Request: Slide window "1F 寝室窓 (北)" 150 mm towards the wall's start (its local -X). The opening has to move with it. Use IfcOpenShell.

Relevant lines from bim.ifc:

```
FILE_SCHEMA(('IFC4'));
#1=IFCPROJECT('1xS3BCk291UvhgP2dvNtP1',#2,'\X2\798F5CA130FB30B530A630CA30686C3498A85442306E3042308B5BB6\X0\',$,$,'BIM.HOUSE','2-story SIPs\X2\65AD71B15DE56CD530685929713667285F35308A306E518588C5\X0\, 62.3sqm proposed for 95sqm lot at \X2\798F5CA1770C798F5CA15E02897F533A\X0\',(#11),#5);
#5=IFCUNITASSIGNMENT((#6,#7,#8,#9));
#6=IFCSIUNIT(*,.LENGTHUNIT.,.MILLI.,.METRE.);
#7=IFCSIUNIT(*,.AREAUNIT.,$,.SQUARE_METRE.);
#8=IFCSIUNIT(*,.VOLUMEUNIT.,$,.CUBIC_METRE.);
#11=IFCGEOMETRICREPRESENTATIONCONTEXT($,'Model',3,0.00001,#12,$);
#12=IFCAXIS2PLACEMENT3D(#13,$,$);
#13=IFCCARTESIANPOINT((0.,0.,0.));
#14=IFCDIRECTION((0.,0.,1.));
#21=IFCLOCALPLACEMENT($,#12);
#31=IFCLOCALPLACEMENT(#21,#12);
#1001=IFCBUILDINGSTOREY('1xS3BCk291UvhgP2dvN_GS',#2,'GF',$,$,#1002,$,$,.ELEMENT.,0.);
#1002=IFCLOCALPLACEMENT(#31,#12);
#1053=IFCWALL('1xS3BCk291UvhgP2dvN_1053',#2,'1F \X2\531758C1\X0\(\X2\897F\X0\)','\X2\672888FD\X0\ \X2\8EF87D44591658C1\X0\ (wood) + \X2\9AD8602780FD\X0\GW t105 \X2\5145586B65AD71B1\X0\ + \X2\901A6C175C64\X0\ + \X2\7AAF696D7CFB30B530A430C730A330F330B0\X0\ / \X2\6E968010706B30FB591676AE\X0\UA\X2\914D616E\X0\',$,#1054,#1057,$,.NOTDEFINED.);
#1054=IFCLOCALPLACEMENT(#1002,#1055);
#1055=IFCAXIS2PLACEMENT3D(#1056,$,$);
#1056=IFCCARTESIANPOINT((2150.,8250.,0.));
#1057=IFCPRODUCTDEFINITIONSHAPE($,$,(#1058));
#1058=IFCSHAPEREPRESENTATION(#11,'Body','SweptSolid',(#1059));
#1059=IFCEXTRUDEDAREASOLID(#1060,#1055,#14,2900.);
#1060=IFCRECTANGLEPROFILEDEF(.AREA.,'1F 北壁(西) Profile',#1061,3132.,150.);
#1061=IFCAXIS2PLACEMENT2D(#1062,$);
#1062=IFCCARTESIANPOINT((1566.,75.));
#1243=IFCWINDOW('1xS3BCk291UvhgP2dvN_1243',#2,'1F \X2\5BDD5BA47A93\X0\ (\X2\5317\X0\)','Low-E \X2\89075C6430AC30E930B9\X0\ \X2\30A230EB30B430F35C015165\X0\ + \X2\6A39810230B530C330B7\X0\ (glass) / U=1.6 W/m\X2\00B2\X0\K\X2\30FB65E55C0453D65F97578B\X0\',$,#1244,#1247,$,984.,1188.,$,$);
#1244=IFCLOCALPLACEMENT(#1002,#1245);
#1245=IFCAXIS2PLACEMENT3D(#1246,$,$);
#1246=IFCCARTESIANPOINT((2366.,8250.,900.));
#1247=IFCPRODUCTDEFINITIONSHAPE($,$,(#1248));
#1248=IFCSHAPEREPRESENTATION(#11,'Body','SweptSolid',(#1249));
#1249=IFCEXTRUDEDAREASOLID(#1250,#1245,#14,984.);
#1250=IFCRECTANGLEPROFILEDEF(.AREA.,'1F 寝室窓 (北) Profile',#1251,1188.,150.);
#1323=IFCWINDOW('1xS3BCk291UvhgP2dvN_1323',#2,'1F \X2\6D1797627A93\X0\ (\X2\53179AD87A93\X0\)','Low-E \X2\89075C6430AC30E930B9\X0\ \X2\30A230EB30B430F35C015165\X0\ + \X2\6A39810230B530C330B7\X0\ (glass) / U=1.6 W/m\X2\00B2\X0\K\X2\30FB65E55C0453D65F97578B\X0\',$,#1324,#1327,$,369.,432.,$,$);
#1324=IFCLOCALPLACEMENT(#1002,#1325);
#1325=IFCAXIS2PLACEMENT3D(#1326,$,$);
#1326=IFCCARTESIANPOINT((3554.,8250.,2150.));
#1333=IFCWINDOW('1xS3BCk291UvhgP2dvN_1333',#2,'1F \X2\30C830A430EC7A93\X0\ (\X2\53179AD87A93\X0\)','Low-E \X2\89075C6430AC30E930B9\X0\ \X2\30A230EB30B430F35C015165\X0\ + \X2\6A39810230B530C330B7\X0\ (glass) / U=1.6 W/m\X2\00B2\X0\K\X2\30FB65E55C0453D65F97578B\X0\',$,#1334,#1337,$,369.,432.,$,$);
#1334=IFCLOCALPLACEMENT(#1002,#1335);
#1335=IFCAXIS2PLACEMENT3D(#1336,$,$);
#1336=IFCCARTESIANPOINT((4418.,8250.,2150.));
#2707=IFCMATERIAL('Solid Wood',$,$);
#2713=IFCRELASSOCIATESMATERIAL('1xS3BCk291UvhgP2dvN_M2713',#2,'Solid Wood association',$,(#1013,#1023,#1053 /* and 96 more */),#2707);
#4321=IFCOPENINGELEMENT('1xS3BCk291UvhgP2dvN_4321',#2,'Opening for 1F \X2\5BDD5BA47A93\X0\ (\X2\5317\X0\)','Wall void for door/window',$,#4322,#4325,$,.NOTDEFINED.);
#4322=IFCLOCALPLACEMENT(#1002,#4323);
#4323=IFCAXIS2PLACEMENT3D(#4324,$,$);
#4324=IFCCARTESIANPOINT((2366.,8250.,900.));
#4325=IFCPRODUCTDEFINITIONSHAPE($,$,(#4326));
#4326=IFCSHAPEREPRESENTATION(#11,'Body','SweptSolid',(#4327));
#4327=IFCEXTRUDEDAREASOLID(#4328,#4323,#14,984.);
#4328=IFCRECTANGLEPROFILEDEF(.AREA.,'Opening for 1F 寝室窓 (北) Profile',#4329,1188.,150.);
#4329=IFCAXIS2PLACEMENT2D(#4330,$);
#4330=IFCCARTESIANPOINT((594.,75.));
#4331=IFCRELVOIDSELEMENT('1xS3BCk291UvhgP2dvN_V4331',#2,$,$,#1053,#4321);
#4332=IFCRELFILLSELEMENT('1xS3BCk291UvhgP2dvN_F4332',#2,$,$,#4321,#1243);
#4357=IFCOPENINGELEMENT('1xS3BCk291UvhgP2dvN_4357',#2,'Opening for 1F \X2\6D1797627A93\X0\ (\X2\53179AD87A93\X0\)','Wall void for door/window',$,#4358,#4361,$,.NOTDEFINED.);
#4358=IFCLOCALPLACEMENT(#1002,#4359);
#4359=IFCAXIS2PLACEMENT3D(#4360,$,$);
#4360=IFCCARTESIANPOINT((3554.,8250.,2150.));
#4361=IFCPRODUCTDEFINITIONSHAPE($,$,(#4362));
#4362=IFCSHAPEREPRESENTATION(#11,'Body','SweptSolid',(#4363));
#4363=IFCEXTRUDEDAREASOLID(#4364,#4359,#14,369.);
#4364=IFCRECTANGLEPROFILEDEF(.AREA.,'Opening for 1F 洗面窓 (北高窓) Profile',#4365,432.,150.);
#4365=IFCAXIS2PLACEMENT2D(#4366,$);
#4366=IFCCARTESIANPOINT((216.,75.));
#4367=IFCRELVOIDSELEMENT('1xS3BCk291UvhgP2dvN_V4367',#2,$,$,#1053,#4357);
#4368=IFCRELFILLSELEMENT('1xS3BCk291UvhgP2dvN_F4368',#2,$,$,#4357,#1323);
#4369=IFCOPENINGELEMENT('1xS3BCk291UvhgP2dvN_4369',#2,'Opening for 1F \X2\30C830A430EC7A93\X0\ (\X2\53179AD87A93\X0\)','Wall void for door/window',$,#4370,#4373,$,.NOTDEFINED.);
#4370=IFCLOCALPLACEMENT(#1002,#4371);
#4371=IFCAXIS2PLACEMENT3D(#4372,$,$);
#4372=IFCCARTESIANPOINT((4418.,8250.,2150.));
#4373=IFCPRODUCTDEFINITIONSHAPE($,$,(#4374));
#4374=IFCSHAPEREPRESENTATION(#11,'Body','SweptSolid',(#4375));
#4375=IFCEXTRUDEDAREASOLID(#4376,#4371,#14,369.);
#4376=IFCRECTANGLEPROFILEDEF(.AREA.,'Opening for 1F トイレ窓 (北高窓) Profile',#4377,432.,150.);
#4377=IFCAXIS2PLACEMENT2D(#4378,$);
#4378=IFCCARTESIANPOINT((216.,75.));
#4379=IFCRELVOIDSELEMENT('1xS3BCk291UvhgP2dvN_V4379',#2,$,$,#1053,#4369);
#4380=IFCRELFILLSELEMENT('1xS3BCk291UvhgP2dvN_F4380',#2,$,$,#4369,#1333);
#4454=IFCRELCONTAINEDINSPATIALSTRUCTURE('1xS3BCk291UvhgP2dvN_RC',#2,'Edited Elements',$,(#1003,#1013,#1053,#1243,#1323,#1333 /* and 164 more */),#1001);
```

```python
import ifcopenshell
import ifcopenshell.api.geometry
import ifcopenshell.util.placement

model = ifcopenshell.open("bim.ifc")

window = model.by_guid("1xS3BCk291UvhgP2dvN_1243")
opening = window.FillsVoids[0].RelatingOpeningElement
wall = opening.VoidsElements[0].RelatingBuildingElement

wall_matrix = ifcopenshell.util.placement.get_local_placement(wall.ObjectPlacement)
shift = wall_matrix[:3, 0] * -150.0
before = ifcopenshell.util.placement.get_local_placement(window.ObjectPlacement)[:3, 3].copy()

# The window is not placed relative to its opening, so move both.
for product in (opening, window):
    matrix = ifcopenshell.util.placement.get_local_placement(product.ObjectPlacement)
    matrix[:3, 3] += shift
    ifcopenshell.api.geometry.edit_object_placement(model, product=product, matrix=matrix, is_si=False)

after = ifcopenshell.util.placement.get_local_placement(window.ObjectPlacement)[:3, 3]
print("window moved by", (after - before).round(3) + 0.0)

model.write("bim-out.ifc")
```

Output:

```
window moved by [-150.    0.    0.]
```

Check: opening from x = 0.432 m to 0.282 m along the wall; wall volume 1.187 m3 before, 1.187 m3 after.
